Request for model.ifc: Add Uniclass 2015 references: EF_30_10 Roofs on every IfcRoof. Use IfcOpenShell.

First a look at what the model holds.

```python
import ifcopenshell

model = ifcopenshell.open("model.ifc")
print(model.schema)
print("classifications:", [c.Name for c in model.by_type("IfcClassification")])
for ifc_class in ("IfcDoor", "IfcRoof", "IfcStair", "IfcWall", "IfcWindow"):
    print(ifc_class, len(model.by_type(ifc_class)))
```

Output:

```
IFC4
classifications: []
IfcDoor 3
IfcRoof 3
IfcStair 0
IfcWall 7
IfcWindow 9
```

```python
import ifcopenshell
import ifcopenshell.api.classification

model = ifcopenshell.open("model.ifc")

system = ifcopenshell.api.classification.add_classification(model, classification="Uniclass 2015")

codes = {
    "IfcRoof": ("EF_30_10", "Roofs"),
}
for ifc_class, (code, name) in codes.items():
    products = model.by_type(ifc_class)
    ifcopenshell.api.classification.add_reference(
        model, products=products, classification=system, identification=code, name=name
    )
    print(code, len(products))

model.write("model_updated.ifc")
```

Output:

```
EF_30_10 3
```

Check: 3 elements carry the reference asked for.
